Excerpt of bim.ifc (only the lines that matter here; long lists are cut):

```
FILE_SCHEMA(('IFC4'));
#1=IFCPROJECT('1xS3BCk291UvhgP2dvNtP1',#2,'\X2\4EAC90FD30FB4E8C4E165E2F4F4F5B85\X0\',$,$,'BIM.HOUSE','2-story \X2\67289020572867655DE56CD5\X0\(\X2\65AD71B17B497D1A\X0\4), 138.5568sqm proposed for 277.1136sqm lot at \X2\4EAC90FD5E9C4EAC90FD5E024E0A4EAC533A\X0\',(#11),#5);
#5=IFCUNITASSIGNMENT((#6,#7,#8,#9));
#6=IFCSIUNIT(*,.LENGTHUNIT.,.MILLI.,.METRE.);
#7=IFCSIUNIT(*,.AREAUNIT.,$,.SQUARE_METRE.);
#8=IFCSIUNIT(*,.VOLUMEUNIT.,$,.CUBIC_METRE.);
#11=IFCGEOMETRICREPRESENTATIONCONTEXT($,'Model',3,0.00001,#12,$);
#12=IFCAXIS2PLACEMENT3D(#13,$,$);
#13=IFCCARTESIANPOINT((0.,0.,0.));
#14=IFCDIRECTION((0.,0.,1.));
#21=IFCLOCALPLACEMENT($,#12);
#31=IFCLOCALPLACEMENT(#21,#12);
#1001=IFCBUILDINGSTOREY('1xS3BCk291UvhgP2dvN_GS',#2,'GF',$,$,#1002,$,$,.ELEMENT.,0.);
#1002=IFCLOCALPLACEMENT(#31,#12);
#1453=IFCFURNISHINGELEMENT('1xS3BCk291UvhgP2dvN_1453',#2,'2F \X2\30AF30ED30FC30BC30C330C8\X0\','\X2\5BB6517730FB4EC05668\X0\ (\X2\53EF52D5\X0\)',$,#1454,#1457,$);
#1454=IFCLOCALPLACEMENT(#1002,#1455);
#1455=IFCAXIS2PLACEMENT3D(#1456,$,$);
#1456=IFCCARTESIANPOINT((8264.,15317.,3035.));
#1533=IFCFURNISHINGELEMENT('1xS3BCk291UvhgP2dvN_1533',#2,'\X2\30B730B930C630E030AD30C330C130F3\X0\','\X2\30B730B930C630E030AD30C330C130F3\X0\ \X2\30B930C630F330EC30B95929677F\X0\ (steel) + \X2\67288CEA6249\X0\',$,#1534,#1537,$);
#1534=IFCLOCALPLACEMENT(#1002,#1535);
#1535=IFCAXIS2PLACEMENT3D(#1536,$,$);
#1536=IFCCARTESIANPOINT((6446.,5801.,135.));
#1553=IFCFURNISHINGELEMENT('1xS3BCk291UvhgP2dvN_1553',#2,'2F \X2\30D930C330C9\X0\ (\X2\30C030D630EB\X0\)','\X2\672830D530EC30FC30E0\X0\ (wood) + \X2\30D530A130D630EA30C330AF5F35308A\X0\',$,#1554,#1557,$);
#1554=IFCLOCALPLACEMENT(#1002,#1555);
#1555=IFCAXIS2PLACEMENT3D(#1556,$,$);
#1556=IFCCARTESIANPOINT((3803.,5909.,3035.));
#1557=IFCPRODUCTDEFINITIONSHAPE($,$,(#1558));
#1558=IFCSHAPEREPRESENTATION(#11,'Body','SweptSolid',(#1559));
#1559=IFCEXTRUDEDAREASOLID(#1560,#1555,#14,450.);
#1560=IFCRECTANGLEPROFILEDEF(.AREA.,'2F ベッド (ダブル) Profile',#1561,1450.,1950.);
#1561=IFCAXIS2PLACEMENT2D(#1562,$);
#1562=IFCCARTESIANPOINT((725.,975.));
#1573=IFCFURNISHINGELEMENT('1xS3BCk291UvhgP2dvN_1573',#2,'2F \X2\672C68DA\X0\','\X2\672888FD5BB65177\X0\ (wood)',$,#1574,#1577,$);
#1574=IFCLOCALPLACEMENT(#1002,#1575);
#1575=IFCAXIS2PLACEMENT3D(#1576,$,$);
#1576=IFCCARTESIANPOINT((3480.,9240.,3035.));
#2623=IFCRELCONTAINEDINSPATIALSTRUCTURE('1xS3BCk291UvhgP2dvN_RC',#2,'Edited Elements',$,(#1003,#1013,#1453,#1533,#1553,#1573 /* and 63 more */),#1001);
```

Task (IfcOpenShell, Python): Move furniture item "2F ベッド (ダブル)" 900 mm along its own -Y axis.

```python
import ifcopenshell
import ifcopenshell.api.geometry
import ifcopenshell.util.placement

model = ifcopenshell.open("bim.ifc")

item = model.by_guid("1xS3BCk291UvhgP2dvN_1553")
matrix = ifcopenshell.util.placement.get_local_placement(item.ObjectPlacement)
matrix[:3, 3] -= matrix[:3, 1] * 900.0
ifcopenshell.api.geometry.edit_object_placement(model, product=item, matrix=matrix, is_si=False)

print(ifcopenshell.util.placement.get_local_placement(item.ObjectPlacement).round(3) + 0.0)

model.write("bim_edited.ifc")
```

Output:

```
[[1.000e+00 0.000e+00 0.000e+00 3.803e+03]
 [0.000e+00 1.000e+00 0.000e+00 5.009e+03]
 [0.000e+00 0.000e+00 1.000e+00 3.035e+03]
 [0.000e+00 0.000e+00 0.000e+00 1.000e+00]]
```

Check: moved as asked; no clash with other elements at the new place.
